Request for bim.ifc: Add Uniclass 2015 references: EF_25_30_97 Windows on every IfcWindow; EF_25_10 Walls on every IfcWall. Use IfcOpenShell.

First a look at what the model holds.

```python
import ifcopenshell

model = ifcopenshell.open("bim.ifc")
print(model.schema)
print("classifications:", [c.Name for c in model.by_type("IfcClassification")])
for ifc_class in ("IfcDoor", "IfcRoof", "IfcStair", "IfcWall", "IfcWindow"):
    print(ifc_class, len(model.by_type(ifc_class)))
```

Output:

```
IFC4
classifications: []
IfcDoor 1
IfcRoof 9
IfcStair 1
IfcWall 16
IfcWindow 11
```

```python
import ifcopenshell
import ifcopenshell.api.classification

model = ifcopenshell.open("bim.ifc")

system = ifcopenshell.api.classification.add_classification(model, classification="Uniclass 2015")

codes = {
    "IfcWindow": ("EF_25_30_97", "Windows"),
    "IfcWall": ("EF_25_10", "Walls"),
}
for ifc_class, (code, name) in codes.items():
    products = model.by_type(ifc_class)
    ifcopenshell.api.classification.add_reference(
        model, products=products, classification=system, identification=code, name=name
    )
    print(code, len(products))

model.write("bim_edited.ifc")
```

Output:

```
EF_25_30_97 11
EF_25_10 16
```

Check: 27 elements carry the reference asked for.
